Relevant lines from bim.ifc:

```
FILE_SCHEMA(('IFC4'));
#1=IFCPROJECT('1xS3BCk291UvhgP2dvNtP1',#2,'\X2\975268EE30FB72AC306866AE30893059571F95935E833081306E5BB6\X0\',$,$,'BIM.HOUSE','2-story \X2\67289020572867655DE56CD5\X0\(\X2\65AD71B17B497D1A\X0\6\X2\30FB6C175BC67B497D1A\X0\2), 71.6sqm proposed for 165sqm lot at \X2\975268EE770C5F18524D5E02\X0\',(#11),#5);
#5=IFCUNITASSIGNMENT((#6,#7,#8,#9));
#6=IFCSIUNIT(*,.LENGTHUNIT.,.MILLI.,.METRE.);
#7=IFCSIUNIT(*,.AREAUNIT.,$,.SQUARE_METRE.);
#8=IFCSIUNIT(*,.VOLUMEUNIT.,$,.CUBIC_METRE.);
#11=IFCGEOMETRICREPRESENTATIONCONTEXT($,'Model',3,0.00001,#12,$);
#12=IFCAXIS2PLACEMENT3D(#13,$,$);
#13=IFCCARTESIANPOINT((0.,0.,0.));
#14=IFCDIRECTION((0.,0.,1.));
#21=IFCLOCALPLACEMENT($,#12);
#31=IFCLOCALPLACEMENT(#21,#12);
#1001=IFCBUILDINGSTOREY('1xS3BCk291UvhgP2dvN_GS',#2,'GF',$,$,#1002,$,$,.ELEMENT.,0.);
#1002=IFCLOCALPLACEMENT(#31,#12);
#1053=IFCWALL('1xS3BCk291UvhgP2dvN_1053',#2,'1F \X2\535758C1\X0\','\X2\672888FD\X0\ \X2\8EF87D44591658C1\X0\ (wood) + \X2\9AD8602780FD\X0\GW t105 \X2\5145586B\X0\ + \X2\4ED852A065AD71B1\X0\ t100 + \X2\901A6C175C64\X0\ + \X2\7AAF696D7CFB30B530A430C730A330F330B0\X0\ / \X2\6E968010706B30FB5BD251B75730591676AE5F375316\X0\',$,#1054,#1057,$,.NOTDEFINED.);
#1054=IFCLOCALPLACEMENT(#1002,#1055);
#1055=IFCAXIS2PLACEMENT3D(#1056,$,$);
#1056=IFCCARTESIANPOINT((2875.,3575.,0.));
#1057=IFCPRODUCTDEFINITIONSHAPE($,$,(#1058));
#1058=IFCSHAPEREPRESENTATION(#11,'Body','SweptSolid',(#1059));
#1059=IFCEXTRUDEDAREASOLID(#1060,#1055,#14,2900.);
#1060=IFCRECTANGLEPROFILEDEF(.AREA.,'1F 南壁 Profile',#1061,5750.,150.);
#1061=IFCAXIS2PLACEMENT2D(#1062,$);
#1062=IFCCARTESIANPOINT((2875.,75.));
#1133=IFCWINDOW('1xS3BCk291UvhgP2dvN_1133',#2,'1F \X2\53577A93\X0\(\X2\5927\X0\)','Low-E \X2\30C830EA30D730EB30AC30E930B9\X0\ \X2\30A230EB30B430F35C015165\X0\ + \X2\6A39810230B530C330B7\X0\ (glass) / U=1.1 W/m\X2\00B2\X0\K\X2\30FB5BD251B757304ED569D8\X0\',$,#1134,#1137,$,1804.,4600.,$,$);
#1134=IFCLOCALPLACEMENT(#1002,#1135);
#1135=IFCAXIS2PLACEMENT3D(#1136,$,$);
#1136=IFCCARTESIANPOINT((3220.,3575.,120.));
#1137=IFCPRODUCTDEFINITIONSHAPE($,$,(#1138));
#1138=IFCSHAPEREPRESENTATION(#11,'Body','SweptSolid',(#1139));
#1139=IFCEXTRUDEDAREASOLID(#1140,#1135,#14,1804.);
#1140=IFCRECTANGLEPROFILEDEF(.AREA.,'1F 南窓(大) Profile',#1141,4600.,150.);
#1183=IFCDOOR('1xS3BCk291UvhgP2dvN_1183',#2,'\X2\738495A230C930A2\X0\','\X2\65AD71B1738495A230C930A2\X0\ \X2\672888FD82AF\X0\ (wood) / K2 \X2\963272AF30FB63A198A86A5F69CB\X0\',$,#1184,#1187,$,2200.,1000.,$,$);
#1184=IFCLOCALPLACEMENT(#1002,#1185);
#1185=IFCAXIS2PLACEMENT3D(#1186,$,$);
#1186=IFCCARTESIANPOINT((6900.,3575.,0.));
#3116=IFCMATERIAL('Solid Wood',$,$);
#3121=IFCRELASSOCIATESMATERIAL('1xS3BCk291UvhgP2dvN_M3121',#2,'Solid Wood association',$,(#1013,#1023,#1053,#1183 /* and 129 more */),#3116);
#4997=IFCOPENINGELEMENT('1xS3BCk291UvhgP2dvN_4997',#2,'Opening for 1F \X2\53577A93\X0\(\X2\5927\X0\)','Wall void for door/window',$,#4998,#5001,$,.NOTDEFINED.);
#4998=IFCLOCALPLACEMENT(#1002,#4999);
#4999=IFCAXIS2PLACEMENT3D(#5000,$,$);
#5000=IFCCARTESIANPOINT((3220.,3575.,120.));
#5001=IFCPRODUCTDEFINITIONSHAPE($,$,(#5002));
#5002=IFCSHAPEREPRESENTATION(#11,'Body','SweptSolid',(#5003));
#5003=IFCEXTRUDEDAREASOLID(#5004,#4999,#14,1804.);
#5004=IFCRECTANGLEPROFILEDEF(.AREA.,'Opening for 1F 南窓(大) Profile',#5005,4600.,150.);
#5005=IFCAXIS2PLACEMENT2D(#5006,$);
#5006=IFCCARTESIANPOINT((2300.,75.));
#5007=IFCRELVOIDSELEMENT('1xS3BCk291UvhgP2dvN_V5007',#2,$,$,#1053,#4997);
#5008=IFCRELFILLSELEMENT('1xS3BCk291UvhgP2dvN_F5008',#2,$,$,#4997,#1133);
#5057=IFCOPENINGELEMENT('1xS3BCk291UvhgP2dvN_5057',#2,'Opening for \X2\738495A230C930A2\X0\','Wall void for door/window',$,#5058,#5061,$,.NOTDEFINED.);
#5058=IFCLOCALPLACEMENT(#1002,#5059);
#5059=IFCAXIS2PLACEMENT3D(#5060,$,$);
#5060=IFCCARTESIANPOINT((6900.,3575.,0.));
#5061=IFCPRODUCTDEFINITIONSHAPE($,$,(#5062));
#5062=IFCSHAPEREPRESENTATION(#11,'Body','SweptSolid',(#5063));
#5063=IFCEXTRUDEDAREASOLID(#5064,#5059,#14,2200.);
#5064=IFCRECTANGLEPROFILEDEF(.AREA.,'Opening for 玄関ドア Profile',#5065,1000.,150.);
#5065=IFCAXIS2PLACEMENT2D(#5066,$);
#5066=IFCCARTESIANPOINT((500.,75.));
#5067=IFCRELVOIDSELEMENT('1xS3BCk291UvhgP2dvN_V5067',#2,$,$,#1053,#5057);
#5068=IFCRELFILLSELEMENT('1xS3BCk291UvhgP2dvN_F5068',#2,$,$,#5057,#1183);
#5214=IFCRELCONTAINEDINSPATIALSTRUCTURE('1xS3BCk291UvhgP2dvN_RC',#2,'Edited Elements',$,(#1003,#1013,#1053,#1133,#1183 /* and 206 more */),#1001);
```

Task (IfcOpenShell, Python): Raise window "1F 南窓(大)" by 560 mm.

```python
import numpy as np
import ifcopenshell
import ifcopenshell.api.geometry
import ifcopenshell.util.placement
import ifcopenshell.util.unit

model = ifcopenshell.open("bim.ifc")
unit_scale = ifcopenshell.util.unit.calculate_unit_scale(model)

window = model.by_id(1133)
opening = window.FillsVoids[0].RelatingOpeningElement
dz = 0.56 / unit_scale

shift = np.array([0.0, 0.0, dz])
# The window is not placed relative to its opening, so move both.
for product in (opening, window):
    matrix = ifcopenshell.util.placement.get_local_placement(product.ObjectPlacement)
    matrix[:3, 3] += shift
    ifcopenshell.api.geometry.edit_object_placement(model, product=product, matrix=matrix, is_si=False)

print(f"moved by {dz * unit_scale:+.3f} m")

model.write("bim_v2.ifc")
```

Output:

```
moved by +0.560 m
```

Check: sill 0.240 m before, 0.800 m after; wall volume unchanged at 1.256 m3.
